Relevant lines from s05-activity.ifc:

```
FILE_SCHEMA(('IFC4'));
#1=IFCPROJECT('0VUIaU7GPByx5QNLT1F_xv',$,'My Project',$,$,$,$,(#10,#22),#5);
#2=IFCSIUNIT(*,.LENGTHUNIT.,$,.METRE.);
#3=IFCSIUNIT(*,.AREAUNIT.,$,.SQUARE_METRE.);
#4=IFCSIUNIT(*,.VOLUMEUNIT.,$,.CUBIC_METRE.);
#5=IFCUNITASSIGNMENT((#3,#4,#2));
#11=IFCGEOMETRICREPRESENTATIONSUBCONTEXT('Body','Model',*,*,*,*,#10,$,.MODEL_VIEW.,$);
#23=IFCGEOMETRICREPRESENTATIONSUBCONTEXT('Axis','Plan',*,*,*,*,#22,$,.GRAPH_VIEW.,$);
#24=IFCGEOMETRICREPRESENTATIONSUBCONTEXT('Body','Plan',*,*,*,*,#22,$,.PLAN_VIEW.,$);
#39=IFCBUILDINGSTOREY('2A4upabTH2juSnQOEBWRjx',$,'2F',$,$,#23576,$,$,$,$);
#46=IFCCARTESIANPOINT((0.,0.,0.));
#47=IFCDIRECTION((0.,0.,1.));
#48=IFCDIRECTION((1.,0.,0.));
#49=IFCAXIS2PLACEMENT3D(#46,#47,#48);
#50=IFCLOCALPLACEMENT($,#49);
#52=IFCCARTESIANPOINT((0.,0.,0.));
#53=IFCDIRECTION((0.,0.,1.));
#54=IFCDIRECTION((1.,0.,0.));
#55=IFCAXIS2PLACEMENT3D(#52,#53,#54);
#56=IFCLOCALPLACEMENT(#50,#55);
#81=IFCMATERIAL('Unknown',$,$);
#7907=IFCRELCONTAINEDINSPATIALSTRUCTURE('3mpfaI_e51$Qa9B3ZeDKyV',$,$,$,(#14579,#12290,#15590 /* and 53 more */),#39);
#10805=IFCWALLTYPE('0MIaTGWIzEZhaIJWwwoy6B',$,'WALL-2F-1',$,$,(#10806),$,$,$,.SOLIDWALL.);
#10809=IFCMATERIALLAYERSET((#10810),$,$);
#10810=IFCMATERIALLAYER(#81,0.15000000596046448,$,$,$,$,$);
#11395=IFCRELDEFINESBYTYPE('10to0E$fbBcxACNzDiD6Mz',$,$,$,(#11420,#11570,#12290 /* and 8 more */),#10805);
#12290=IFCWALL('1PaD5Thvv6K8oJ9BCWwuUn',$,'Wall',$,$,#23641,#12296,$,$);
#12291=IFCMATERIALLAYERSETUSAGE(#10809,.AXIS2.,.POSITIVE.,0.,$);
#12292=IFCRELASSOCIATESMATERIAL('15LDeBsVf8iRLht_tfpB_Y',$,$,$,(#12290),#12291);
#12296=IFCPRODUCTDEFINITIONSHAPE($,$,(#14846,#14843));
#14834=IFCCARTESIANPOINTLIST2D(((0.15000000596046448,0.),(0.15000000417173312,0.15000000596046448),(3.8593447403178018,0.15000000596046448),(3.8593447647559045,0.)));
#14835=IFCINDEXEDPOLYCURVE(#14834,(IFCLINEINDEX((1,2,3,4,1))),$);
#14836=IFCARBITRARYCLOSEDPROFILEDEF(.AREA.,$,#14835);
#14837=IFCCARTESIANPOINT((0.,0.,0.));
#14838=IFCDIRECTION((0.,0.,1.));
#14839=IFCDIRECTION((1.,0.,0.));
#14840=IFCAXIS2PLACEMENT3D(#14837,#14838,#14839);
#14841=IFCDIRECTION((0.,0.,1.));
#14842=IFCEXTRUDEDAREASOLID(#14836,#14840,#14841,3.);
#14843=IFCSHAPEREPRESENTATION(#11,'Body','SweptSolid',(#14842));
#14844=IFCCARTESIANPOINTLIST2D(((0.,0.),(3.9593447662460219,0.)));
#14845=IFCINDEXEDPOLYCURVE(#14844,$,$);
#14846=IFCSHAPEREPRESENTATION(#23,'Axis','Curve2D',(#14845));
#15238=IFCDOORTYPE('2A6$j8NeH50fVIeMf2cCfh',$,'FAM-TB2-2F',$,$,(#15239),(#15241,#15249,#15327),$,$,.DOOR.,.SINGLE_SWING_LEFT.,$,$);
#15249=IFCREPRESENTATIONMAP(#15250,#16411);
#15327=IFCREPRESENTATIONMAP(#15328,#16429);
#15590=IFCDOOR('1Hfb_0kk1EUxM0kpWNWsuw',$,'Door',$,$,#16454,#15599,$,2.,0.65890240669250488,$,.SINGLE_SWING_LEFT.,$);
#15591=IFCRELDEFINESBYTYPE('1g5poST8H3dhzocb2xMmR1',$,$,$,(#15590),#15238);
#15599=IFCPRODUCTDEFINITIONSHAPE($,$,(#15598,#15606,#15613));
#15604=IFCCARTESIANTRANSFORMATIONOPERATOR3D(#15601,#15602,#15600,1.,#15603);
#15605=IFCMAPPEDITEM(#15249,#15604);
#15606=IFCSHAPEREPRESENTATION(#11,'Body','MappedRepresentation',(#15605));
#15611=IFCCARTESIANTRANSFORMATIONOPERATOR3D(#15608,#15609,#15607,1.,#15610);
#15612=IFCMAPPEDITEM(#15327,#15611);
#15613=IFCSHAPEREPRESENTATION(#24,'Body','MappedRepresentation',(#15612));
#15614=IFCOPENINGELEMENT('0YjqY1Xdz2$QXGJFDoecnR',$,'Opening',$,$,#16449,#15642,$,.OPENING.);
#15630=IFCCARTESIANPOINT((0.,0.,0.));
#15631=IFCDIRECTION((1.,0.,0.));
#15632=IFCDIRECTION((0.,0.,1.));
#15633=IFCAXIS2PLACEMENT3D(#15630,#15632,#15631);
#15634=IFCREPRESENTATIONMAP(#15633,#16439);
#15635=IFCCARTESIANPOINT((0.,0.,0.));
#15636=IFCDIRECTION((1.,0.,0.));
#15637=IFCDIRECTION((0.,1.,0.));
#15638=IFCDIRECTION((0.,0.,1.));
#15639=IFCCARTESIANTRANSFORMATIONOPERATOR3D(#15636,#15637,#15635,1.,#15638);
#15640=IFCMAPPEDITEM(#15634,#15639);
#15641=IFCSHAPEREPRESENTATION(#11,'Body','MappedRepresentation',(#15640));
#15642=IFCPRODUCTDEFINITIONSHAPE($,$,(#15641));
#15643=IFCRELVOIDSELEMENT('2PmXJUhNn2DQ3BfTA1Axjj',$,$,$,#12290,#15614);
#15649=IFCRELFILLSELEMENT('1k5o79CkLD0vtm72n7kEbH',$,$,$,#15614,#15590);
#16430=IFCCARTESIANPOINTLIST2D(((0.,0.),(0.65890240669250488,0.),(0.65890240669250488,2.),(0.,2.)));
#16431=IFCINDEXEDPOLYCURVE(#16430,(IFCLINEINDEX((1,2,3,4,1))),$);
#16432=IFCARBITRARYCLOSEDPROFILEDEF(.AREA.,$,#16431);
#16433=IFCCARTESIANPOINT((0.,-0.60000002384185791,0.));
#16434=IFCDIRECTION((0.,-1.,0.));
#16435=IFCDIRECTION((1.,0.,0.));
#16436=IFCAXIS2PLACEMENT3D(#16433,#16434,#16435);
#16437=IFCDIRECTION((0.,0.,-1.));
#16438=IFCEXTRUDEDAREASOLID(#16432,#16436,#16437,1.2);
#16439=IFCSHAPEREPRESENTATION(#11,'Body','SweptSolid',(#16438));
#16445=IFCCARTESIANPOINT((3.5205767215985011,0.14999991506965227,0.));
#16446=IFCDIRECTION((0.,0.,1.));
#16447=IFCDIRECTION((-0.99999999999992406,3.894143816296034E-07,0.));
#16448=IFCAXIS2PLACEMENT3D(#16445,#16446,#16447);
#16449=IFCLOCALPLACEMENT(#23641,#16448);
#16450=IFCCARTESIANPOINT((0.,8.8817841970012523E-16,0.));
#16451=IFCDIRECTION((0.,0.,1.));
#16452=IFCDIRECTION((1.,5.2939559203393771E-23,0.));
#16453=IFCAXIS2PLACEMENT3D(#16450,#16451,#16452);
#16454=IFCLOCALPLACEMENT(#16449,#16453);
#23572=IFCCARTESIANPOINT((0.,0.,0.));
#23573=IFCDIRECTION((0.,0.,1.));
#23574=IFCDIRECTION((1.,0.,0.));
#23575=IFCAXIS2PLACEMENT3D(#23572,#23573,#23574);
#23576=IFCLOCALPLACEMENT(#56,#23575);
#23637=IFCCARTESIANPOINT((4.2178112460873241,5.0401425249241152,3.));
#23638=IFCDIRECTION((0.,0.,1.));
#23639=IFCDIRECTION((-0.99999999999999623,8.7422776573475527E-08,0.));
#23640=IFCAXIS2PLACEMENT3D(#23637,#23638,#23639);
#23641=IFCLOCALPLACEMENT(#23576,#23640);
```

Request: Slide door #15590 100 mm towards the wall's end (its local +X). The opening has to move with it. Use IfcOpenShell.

```python
import ifcopenshell
import ifcopenshell.api.geometry
import ifcopenshell.util.placement
import ifcopenshell.util.unit

model = ifcopenshell.open("s05-activity.ifc")
unit_scale = ifcopenshell.util.unit.calculate_unit_scale(model)

door = model.by_guid("1Hfb_0kk1EUxM0kpWNWsuw")
opening = door.FillsVoids[0].RelatingOpeningElement
wall = opening.VoidsElements[0].RelatingBuildingElement

wall_matrix = ifcopenshell.util.placement.get_local_placement(wall.ObjectPlacement)
shift = wall_matrix[:3, 0] * 0.1 / unit_scale
before = ifcopenshell.util.placement.get_local_placement(door.ObjectPlacement)[:3, 3].copy()

# The door is placed relative to its opening, so it follows when the opening moves.
matrix = ifcopenshell.util.placement.get_local_placement(opening.ObjectPlacement)
matrix[:3, 3] += shift
ifcopenshell.api.geometry.edit_object_placement(
    model, product=opening, matrix=matrix, is_si=False, should_transform_children=True
)

after = ifcopenshell.util.placement.get_local_placement(door.ObjectPlacement)[:3, 3]
print("door moved by", (after - before).round(3) + 0.0)

model.write("s05-activity-out.ifc")
```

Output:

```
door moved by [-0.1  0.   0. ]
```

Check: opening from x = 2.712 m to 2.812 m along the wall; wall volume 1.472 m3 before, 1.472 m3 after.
